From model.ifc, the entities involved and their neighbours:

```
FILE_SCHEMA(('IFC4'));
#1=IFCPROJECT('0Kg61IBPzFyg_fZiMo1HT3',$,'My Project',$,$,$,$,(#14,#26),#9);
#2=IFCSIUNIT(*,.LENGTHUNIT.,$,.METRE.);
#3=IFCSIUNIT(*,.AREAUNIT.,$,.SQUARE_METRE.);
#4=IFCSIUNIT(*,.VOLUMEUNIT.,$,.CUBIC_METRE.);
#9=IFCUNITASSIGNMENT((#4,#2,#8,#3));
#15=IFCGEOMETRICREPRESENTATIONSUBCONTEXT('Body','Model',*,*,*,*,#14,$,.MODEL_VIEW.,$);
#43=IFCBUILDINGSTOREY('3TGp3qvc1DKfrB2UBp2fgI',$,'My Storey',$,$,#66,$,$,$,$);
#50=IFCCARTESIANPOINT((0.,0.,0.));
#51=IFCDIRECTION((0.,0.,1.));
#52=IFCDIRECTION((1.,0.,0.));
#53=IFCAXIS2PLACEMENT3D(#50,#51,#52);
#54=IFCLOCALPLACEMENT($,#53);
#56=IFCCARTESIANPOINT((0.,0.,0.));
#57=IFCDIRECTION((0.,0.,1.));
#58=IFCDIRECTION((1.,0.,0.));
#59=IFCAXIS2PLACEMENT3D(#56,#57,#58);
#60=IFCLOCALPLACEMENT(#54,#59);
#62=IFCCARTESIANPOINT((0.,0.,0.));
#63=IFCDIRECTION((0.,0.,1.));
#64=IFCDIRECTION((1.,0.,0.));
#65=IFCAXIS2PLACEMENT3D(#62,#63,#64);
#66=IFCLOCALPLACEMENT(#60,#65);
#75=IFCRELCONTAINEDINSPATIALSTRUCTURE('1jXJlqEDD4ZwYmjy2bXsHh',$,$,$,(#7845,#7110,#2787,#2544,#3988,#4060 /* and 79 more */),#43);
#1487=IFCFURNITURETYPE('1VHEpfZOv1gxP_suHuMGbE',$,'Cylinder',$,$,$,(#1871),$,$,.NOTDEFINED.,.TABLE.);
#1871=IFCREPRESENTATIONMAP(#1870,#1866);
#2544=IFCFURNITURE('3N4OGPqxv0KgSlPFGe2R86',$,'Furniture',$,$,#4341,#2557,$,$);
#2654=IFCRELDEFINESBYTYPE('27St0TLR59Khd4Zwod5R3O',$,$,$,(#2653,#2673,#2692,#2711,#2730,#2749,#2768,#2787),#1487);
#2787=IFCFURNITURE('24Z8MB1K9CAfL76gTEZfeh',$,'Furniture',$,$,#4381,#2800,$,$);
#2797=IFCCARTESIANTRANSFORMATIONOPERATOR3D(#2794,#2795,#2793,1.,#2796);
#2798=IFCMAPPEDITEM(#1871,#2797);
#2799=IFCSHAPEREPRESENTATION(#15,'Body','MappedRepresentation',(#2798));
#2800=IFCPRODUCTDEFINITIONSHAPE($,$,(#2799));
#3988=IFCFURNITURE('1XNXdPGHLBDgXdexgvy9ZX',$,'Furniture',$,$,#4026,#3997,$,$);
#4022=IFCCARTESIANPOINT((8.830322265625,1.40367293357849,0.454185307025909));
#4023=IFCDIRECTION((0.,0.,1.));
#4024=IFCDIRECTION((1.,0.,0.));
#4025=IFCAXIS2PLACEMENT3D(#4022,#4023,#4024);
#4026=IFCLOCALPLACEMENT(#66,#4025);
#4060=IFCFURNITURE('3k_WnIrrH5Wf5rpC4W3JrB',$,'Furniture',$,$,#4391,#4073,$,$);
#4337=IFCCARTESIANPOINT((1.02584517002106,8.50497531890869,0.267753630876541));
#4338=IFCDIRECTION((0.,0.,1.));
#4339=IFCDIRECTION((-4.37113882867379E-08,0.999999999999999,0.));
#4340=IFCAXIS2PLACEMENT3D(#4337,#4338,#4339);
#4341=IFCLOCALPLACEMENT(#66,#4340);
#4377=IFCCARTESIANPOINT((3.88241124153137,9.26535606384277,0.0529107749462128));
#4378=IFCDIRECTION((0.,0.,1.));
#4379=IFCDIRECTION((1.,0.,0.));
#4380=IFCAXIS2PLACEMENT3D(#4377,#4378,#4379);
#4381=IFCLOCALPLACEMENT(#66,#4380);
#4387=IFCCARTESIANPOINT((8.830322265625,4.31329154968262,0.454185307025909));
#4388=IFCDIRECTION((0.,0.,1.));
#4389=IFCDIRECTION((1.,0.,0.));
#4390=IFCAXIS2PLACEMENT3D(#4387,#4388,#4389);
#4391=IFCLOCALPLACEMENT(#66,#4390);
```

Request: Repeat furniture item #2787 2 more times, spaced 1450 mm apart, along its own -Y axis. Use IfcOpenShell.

```python
import ifcopenshell
import ifcopenshell.api.geometry
import ifcopenshell.api.root
import ifcopenshell.util.element
import ifcopenshell.util.placement
import ifcopenshell.util.unit

model = ifcopenshell.open("model.ifc")
unit_scale = ifcopenshell.util.unit.calculate_unit_scale(model)

source = model.by_id(2787)
base = ifcopenshell.util.placement.get_local_placement(source.ObjectPlacement)
step = -base[:3, 1] * 1.45 / unit_scale

for i in range(1, 3):
    copy = ifcopenshell.api.root.copy_class(model, product=source)
    copy.Representation = ifcopenshell.util.element.copy_deep(
        model, source.Representation, exclude=["IfcGeometricRepresentationContext", "IfcRepresentationMap"]
    )
    matrix = base.copy()
    matrix[:3, 3] += i * step
    print("added at", matrix[:3, 3].round(3) + 0.0)
    ifcopenshell.api.geometry.edit_object_placement(model, product=copy, matrix=matrix, is_si=False)

model.write("model_edited.ifc")
```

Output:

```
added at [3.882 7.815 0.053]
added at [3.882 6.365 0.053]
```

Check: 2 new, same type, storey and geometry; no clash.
